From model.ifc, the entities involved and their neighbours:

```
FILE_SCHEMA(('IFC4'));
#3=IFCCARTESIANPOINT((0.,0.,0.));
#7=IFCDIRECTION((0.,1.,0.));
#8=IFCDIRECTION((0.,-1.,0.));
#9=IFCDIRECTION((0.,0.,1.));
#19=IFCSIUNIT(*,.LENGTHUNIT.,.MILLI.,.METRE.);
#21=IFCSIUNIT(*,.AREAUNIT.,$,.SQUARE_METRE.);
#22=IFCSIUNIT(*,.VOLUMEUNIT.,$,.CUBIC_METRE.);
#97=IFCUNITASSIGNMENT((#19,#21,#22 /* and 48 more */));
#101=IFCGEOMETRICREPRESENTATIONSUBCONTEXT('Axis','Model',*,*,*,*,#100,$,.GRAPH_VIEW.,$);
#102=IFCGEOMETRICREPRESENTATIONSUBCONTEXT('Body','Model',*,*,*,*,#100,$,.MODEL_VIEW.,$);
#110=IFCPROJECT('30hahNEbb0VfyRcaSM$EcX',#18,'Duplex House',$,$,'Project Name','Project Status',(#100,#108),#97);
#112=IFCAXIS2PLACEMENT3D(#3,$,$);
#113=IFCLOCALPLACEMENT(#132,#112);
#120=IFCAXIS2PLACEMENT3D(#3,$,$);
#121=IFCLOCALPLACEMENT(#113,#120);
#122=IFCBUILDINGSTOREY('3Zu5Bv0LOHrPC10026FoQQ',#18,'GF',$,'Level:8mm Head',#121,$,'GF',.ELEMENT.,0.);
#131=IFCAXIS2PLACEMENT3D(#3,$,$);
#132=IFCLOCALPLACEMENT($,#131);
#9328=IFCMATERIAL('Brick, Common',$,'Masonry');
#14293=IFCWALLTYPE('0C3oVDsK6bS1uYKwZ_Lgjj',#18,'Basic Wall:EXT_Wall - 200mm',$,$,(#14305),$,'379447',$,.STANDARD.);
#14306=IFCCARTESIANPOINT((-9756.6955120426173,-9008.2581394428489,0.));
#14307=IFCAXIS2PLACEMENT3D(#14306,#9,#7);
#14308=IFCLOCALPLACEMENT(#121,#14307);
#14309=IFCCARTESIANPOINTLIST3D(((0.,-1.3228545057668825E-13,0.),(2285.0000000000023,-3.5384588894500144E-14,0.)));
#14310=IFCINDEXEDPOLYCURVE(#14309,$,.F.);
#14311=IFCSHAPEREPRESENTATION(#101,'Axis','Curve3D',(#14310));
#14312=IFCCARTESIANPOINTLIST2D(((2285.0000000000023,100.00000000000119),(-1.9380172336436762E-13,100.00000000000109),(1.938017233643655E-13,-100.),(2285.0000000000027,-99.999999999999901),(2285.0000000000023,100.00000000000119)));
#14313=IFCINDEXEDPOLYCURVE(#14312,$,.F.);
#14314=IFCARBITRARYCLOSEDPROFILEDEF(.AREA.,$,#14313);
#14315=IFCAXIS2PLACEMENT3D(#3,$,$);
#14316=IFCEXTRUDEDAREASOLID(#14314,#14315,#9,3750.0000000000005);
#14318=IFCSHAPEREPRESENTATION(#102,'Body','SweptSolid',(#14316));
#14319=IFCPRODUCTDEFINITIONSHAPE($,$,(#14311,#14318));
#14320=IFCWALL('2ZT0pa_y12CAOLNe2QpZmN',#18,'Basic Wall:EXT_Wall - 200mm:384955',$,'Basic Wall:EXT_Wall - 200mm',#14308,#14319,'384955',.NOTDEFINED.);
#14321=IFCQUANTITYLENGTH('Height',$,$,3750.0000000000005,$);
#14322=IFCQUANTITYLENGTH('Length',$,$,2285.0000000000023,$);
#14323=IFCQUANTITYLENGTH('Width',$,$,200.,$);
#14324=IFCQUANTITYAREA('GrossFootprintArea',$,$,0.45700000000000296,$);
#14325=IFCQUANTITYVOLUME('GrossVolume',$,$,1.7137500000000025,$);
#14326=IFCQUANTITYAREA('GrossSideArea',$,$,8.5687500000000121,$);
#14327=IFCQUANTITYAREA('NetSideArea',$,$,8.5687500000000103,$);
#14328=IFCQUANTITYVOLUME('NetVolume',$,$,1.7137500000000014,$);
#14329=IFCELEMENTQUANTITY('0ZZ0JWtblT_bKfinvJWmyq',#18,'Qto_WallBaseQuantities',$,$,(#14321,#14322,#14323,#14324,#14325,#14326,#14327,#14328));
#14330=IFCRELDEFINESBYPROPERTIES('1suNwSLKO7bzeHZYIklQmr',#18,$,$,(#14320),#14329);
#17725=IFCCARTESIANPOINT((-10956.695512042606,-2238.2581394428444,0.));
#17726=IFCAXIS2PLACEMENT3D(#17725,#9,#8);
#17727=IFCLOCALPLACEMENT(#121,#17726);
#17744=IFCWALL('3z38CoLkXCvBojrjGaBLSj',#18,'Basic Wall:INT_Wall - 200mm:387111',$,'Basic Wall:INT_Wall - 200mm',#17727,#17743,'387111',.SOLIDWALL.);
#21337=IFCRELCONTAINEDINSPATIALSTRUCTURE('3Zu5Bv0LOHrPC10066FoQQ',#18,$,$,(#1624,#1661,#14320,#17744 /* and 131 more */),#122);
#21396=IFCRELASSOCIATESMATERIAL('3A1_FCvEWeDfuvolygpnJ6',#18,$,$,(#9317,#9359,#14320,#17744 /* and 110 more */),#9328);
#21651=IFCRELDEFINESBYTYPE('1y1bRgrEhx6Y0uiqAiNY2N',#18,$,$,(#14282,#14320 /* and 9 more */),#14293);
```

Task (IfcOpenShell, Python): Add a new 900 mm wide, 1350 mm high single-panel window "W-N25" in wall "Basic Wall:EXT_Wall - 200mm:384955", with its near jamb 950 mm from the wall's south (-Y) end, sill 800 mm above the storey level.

```python
import numpy as np
import ifcopenshell
import ifcopenshell.api.feature
import ifcopenshell.api.geometry
import ifcopenshell.api.pset
import ifcopenshell.api.root
import ifcopenshell.api.spatial
import ifcopenshell.geom
import ifcopenshell.util.element
import ifcopenshell.util.placement
import ifcopenshell.util.representation
import ifcopenshell.util.shape
import ifcopenshell.util.unit

model = ifcopenshell.open("model.ifc")
unit_scale = ifcopenshell.util.unit.calculate_unit_scale(model)
area_scale = ifcopenshell.util.unit.calculate_unit_scale(model, "AREAUNIT")
volume_scale = ifcopenshell.util.unit.calculate_unit_scale(model, "VOLUMEUNIT")
settings = ifcopenshell.geom.settings()


def volume(element):
    """Net volume in cubic metres, openings subtracted."""
    shape = ifcopenshell.geom.create_shape(settings, element)
    return ifcopenshell.util.shape.get_volume(shape.geometry)


wall = model.by_guid("2ZT0pa_y12CAOLNe2QpZmN")
storey = ifcopenshell.util.element.get_container(wall, ifc_class="IfcBuildingStorey")
context = ifcopenshell.util.representation.get_context(model, "Model", "Body", "MODEL_VIEW")
before = volume(wall)

width, height, from_end, sill = 0.9, 1.35, 0.95, 0.8  # metres

# The wall runs along its own X axis, and the end named is its -X end.
wall_shape = ifcopenshell.geom.create_shape(settings, wall)
x, y, z = ifcopenshell.util.shape.get_vertices(wall_shape.geometry).T
start = x.min() + from_end
face, thickness = float(y.min()), float(y.max() - y.min())
wall_matrix = ifcopenshell.util.placement.get_local_placement(wall.ObjectPlacement)
level = ifcopenshell.util.placement.get_local_placement(storey.ObjectPlacement)[2, 3]


def in_wall(x, y):
    """Placement at x, y metres in the wall's axes, at sill height."""
    matrix = wall_matrix.copy()
    matrix[:, 3] = wall_matrix @ np.array([x / unit_scale, y / unit_scale, 0.0, 1.0])
    matrix[2, 3] = level + sill / unit_scale
    return matrix


# Opening: a box that overshoots both wall faces by 50 mm.
opening = ifcopenshell.api.root.create_entity(model, ifc_class="IfcOpeningElement", predefined_type="OPENING")
box = ifcopenshell.api.geometry.add_wall_representation(
    model, context=context, length=width, height=height, thickness=thickness + 0.1
)
ifcopenshell.api.geometry.assign_representation(model, product=opening, representation=box)
ifcopenshell.api.geometry.edit_object_placement(model, product=opening, matrix=in_wall(start, face - 0.05), is_si=False)
ifcopenshell.api.feature.add_feature(model, feature=opening, element=wall)

window = ifcopenshell.api.root.create_entity(model, ifc_class="IfcWindow", name="W-N25", predefined_type="WINDOW")
window.OverallWidth, window.OverallHeight = width / unit_scale, height / unit_scale
window.PartitioningType = "SINGLE_PANEL"
body = ifcopenshell.api.geometry.add_window_representation(
    model,
    context=context,
    overall_width=window.OverallWidth,
    overall_height=window.OverallHeight,
    partition_type="SINGLE_PANEL",
)
ifcopenshell.api.geometry.assign_representation(model, product=window, representation=body)
ifcopenshell.api.spatial.assign_container(model, products=[window], relating_structure=storey)
ifcopenshell.api.feature.add_filling(model, opening=opening, element=window)

# Centre the window in the wall's thickness.
ifcopenshell.api.geometry.edit_object_placement(model, product=window, matrix=in_wall(start, face), is_si=False)
window_shape = ifcopenshell.geom.create_shape(settings, window)
depth = ifcopenshell.util.shape.get_vertices(window_shape.geometry)[:, 1]
offset = face + thickness / 2 - (depth.min() + depth.max()) / 2
ifcopenshell.api.geometry.edit_object_placement(model, product=window, matrix=in_wall(start, offset), is_si=False)

after = volume(wall)

# Update the wall's stored quantities.
qto = model.by_id(ifcopenshell.util.element.get_pset(wall, "Qto_WallBaseQuantities", should_inherit=False)["id"])
ifcopenshell.api.pset.edit_qto(model, qto=qto, properties={
    "NetSideArea": after / thickness / area_scale,
    "NetVolume": after / volume_scale,
})

print(f"wall volume {before:.3f} -> {after:.3f} m3")

model.write("model_v2.ifc")
```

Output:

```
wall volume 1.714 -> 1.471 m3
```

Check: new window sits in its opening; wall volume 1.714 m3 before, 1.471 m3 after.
